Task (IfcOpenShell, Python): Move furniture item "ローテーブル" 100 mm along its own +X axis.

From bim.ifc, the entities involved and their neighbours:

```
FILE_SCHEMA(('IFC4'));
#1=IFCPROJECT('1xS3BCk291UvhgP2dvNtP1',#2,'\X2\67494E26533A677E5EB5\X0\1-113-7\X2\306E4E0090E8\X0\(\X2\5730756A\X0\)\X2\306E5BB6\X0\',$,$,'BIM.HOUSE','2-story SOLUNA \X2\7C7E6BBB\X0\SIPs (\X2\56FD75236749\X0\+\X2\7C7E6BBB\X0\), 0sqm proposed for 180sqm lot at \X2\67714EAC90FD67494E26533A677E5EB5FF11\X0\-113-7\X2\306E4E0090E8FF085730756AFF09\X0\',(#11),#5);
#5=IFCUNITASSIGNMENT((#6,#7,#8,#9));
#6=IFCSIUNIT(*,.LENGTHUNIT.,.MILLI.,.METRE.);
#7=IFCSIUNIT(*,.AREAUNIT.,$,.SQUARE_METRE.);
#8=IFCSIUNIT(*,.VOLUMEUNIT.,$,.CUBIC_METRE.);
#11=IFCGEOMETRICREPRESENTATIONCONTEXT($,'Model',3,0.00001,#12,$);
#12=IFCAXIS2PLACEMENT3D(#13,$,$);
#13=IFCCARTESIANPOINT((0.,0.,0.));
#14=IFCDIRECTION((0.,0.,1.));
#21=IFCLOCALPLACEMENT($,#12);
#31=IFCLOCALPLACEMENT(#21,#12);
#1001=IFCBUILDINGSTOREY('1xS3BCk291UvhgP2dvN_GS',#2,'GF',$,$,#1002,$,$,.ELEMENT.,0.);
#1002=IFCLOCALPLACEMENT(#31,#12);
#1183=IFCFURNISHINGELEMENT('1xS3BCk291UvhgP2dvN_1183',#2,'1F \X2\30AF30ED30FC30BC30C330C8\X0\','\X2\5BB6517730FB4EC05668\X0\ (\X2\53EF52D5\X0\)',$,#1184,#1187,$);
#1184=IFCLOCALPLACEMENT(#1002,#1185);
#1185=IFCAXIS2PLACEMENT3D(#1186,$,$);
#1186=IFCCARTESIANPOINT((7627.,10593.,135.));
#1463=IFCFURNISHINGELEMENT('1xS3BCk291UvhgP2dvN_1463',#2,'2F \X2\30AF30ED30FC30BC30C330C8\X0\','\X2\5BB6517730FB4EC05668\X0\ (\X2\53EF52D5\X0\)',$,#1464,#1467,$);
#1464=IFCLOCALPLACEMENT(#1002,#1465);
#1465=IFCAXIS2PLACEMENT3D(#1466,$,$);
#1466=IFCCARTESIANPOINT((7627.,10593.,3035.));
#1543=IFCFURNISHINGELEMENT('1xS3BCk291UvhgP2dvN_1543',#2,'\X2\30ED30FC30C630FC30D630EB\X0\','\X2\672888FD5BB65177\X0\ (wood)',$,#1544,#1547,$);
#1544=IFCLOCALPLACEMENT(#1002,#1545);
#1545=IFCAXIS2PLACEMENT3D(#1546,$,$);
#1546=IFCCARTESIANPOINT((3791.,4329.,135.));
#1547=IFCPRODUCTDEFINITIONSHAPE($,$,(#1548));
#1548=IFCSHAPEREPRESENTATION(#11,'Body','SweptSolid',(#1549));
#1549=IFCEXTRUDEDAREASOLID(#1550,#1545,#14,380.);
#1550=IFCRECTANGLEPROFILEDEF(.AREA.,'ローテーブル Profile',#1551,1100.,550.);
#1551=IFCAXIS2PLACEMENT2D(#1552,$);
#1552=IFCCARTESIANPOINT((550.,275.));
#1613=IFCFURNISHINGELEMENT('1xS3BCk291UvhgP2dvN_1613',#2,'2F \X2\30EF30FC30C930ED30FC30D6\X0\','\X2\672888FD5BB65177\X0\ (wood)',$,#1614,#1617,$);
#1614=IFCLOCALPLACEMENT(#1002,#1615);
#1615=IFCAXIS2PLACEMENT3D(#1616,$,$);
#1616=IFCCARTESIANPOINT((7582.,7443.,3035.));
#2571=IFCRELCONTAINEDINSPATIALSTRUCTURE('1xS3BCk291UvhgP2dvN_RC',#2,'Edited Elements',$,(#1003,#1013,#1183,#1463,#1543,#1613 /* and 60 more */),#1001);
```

```python
import ifcopenshell
import ifcopenshell.api.geometry
import ifcopenshell.util.placement
import ifcopenshell.util.unit

model = ifcopenshell.open("bim.ifc")
unit_scale = ifcopenshell.util.unit.calculate_unit_scale(model)

item = model.by_guid("1xS3BCk291UvhgP2dvN_1543")
matrix = ifcopenshell.util.placement.get_local_placement(item.ObjectPlacement)
matrix[:3, 3] += matrix[:3, 0] * 0.1 / unit_scale
ifcopenshell.api.geometry.edit_object_placement(model, product=item, matrix=matrix, is_si=False)

print(ifcopenshell.util.placement.get_local_placement(item.ObjectPlacement).round(3) + 0.0)

model.write("bim_updated.ifc")
```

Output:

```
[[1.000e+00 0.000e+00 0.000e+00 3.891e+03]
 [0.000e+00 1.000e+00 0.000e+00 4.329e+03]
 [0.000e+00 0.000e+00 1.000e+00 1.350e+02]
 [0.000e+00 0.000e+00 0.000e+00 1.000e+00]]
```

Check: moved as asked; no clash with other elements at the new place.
